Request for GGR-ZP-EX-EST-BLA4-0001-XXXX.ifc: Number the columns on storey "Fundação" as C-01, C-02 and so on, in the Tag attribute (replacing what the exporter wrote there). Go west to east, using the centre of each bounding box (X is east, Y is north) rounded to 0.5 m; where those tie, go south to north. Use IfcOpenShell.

First a look at what the model holds.

```python
import ifcopenshell
import ifcopenshell.util.element
import ifcopenshell.util.placement

model = ifcopenshell.open("GGR-ZP-EX-EST-BLA4-0001-XXXX.ifc")
print(model.schema)
storey = next(s for s in model.by_type("IfcBuildingStorey") if s.Name == "Fundação")
columns = [e for e in ifcopenshell.util.element.get_decomposition(storey) if e.is_a("IfcColumn")]
for e in sorted(columns, key=lambda e: e.id()):
    origin = ifcopenshell.util.placement.get_local_placement(e.ObjectPlacement)[:3, 3]
    print(e.id(), e.Tag, e.Name, origin.round(2) + 0.0, sep=" | ")
```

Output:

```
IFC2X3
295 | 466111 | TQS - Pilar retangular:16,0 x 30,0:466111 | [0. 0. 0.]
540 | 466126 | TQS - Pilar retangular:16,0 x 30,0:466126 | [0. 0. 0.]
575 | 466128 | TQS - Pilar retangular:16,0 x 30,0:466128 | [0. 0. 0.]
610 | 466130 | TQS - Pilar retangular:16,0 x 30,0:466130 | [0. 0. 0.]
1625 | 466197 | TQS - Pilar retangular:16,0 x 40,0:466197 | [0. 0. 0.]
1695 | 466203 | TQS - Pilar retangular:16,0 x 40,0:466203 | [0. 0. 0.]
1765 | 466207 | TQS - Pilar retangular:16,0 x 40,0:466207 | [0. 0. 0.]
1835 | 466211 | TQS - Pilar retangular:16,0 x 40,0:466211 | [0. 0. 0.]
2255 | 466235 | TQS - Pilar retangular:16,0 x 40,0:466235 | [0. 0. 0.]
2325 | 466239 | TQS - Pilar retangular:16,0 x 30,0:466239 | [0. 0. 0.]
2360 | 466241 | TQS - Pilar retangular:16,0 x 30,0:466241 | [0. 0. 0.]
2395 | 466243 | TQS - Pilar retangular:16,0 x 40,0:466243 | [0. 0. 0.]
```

```python
import ifcopenshell
import ifcopenshell.geom
import ifcopenshell.util.element
import ifcopenshell.util.shape

model = ifcopenshell.open("GGR-ZP-EX-EST-BLA4-0001-XXXX.ifc")
settings = ifcopenshell.geom.settings()
settings.set("use-world-coords", True)


def centre(element):
    shape = ifcopenshell.geom.create_shape(settings, element)
    return ifcopenshell.util.shape.get_bbox_centroid(shape.geometry)


storey = next(s for s in model.by_type("IfcBuildingStorey") if s.Name == "Fundação")
columns = [e for e in ifcopenshell.util.element.get_decomposition(storey) if e.is_a("IfcColumn")]

# Insertion points can sit at a corner or the storey origin, so sort by the geometry (in metres).
centres = {e: centre(e) for e in columns}
columns.sort(key=lambda e: (round(centres[e][0] / 0.5), centres[e][1]))

for i, e in enumerate(columns, start=1):
    number = f"C-{i:02d}"
    e.Tag = number
    print(e.id(), number)

model.write("GGR-ZP-EX-EST-BLA4-0001-XXXX_v2.ifc")
```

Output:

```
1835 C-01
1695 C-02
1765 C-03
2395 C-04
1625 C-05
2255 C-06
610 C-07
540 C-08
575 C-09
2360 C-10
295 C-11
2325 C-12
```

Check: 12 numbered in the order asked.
